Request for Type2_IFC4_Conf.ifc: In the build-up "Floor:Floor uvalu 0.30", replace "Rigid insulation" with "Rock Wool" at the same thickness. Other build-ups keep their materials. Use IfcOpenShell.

First a look at what the model holds.

```python
import ifcopenshell
import ifcopenshell.util.element

model = ifcopenshell.open("Type2_IFC4_Conf.ifc")
print(model.schema)
for layer_set in model.by_type("IfcMaterialLayerSet"):
    if layer_set.LayerSetName == "Floor:Floor uvalu 0.30":
        for layer in layer_set.MaterialLayers:
            print(layer.id(), layer.Material and layer.Material.Name, layer.LayerThickness, sep=" | ")
        print(len(ifcopenshell.util.element.get_elements_by_material(model, layer_set)), "elements and types use it")
print(sorted(m.Name for m in model.by_type("IfcMaterial") if m.Name)[:60])
```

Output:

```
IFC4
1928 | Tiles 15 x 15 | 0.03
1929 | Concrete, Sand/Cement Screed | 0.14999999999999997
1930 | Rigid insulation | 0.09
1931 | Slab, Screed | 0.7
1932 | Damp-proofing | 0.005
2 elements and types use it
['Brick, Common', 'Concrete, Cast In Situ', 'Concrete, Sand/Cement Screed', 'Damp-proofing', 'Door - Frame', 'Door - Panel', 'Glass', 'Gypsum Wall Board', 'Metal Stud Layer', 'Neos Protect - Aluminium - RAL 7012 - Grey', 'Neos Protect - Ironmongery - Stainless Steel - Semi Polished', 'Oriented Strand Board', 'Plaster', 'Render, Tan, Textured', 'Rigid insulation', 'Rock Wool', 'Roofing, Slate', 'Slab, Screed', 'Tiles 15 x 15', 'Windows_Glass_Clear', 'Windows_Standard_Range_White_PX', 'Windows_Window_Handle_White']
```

```python
import ifcopenshell
import ifcopenshell.api.material

model = ifcopenshell.open("Type2_IFC4_Conf.ifc")

layer_set = next(s for s in model.by_type("IfcMaterialLayerSet") if s.LayerSetName == "Floor:Floor uvalu 0.30")
layer = next(l for l in layer_set.MaterialLayers if l.Material and l.Material.Name == "Rigid insulation")
material = next(m for m in model.by_type("IfcMaterial") if m.Name == "Rock Wool")

# Point this one layer at the other material; renaming the old one would change it everywhere.
ifcopenshell.api.material.edit_layer(model, layer=layer, attributes={"Name": material.Name}, material=material)

print([l.Material.Name if l.Material else None for l in layer_set.MaterialLayers])

model.write("Type2_IFC4_Conf_v2.ifc")
```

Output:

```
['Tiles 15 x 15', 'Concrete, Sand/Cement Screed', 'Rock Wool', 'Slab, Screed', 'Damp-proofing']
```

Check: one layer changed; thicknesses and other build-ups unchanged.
